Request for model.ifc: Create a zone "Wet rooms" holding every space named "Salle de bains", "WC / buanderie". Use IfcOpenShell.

First a look at what the model holds.

```python
import ifcopenshell

model = ifcopenshell.open("model.ifc")
print(model.schema)
seen = {}
for space in model.by_type("IfcSpace"):
    seen[space.LongName] = seen.get(space.LongName, 0) + 1
for name, count in sorted(seen.items(), key=str):
    print(count, "x", name)
print("zones:", [z.Name for z in model.by_type("IfcZone")][:20])
```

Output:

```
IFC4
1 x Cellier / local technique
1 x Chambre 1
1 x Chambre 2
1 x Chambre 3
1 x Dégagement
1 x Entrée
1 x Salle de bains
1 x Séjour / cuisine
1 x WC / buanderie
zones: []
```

```python
import ifcopenshell
import ifcopenshell.api.group
import ifcopenshell.api.root

model = ifcopenshell.open("model.ifc")

names = {"Salle de bains", "WC / buanderie"}
spaces = [s for s in model.by_type("IfcSpace") if s.LongName in names]

zone = ifcopenshell.api.root.create_entity(model, ifc_class="IfcZone", name="Wet rooms")
ifcopenshell.api.group.assign_group(model, products=spaces, group=zone)
print(len(spaces), "spaces in", zone.Name)

model.write("model_edited.ifc")
```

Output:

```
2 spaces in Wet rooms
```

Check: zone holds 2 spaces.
